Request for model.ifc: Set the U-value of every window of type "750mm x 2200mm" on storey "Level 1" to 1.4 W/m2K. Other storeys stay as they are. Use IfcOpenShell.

First a look at what the model holds.

```python
import ifcopenshell
import ifcopenshell.util.element

model = ifcopenshell.open("model.ifc")
print(model.schema)
storey = next(s for s in model.by_type("IfcBuildingStorey") if s.Name == "Level 1")
windows = [e for e in ifcopenshell.util.element.get_decomposition(storey) if e.is_a("IfcWindow")]
seen = {}
for e in windows:
    element_type = ifcopenshell.util.element.get_type(e)
    key = (element_type.Name if element_type != e and element_type else None, ifcopenshell.util.element.get_pset(e, "Pset_WindowCommon", "ThermalTransmittance"))
    seen[key] = seen.get(key, 0) + 1
for (name, value), count in sorted(seen.items(), key=str):
    print(count, "x", name, "|", value)
```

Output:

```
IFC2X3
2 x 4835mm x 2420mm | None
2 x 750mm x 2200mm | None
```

```python
import ifcopenshell
import ifcopenshell.api.pset
import ifcopenshell.util.element

model = ifcopenshell.open("model.ifc")

storey = next(s for s in model.by_type("IfcBuildingStorey") if s.Name == "Level 1")
windows = [e for e in ifcopenshell.util.element.get_decomposition(storey) if e.is_a("IfcWindow")]

count = 0
for e in windows:
    element_type = ifcopenshell.util.element.get_type(e)
    if element_type in (None, e) or element_type.Name != "750mm x 2200mm":
        continue
    # add_pset returns the element's existing set when there is one.
    pset = ifcopenshell.api.pset.add_pset(model, product=e, name="Pset_WindowCommon")
    ifcopenshell.api.pset.edit_pset(model, pset=pset, properties={"ThermalTransmittance": 1.4})
    count += 1

print(count, "windows updated")

model.write("model_updated.ifc")
```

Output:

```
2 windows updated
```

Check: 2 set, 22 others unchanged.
